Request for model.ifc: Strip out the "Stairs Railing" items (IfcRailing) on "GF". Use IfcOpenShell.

First a look at what the model holds.

```python
import ifcopenshell
import ifcopenshell.util.element

model = ifcopenshell.open("model.ifc")
print(model.schema)
storey = next(s for s in model.by_type("IfcBuildingStorey") if s.Name == "GF")
railings = [e for e in ifcopenshell.util.element.get_decomposition(storey) if e.is_a("IfcRailing")]
seen = {}
for e in railings:
    element_type = ifcopenshell.util.element.get_type(e)
    name = element_type.Name if element_type not in (None, e) else None
    seen[name] = seen.get(name, 0) + 1
for name, count in sorted(seen.items(), key=str):
    print(count, "x", name)
```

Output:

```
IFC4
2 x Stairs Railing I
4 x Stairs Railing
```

```python
import ifcopenshell
import ifcopenshell.api.root
import ifcopenshell.util.element

model = ifcopenshell.open("model.ifc")

storey = next(s for s in model.by_type("IfcBuildingStorey") if s.Name == "GF")
railings = [e for e in ifcopenshell.util.element.get_decomposition(storey) if e.is_a("IfcRailing")]
targets = [e for e in railings if (t := ifcopenshell.util.element.get_type(e)) not in (None, e) and t.Name == "Stairs Railing"]

for e in targets:
    ifcopenshell.api.root.remove_product(model, product=e)
print(len(targets), "removed")

model.write("model-out.ifc")
```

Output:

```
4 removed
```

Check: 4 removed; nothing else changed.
